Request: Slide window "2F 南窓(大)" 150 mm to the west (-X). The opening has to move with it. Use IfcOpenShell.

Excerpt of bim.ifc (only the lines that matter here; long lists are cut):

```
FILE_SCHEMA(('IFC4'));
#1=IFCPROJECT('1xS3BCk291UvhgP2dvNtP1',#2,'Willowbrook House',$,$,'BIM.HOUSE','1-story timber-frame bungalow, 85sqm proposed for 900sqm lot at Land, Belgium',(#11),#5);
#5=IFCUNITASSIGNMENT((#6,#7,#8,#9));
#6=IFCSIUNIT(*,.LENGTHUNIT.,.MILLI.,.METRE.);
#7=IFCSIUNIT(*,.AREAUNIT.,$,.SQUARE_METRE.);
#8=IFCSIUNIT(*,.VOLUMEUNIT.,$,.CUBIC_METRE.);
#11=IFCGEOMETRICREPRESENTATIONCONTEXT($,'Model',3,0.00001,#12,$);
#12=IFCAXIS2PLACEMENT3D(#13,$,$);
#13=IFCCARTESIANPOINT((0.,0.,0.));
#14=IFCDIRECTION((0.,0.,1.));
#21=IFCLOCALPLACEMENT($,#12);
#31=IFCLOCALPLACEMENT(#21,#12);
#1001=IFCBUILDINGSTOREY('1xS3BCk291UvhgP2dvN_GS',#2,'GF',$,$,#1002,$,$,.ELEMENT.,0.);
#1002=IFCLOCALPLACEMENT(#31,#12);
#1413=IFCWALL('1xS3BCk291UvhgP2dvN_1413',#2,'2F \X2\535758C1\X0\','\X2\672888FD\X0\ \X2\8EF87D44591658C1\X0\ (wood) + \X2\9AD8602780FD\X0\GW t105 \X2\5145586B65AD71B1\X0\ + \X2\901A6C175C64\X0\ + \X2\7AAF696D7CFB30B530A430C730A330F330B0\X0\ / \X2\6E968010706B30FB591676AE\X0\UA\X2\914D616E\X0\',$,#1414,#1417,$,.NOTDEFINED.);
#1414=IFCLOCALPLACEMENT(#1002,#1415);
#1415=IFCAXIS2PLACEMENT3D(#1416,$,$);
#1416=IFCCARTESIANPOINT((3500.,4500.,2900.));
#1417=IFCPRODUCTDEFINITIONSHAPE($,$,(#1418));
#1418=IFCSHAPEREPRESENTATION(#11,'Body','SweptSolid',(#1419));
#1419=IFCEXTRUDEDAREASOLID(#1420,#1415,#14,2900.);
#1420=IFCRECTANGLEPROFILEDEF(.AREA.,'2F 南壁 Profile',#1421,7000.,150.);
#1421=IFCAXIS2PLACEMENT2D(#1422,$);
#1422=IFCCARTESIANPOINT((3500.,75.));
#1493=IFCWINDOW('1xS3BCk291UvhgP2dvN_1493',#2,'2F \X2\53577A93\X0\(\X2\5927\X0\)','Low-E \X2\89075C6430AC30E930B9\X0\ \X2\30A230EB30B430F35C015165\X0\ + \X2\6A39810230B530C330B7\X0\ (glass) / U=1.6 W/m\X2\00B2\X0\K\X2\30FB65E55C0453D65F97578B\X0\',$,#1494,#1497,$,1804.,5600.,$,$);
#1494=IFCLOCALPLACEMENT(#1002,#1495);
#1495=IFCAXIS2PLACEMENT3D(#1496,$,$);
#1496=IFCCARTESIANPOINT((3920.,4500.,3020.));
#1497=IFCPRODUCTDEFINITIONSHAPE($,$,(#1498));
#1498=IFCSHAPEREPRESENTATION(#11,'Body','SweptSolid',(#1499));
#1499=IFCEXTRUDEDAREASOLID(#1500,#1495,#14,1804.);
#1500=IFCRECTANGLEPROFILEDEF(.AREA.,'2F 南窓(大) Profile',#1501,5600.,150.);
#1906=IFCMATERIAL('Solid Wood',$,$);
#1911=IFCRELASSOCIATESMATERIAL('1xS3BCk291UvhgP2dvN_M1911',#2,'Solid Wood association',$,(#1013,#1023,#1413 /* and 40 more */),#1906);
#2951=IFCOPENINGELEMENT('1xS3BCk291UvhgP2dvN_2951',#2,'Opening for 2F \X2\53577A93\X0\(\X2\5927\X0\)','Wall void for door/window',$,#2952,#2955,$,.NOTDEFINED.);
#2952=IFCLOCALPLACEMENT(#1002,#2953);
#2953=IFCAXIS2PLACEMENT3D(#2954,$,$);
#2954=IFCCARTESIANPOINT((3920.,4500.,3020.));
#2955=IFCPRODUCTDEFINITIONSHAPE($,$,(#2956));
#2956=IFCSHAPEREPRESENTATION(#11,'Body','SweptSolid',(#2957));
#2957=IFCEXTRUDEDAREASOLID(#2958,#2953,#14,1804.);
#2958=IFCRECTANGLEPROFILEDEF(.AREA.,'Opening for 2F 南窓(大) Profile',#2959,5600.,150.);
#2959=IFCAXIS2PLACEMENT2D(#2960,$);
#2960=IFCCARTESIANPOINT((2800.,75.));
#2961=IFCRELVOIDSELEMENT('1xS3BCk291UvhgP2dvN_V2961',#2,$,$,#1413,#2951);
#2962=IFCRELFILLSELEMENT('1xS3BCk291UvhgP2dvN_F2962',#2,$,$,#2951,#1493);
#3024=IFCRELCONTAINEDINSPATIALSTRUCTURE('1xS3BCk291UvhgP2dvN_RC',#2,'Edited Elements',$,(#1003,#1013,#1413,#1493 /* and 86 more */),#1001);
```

```python
import ifcopenshell
import ifcopenshell.api.geometry
import ifcopenshell.util.placement

model = ifcopenshell.open("bim.ifc")

window = model.by_guid("1xS3BCk291UvhgP2dvN_1493")
opening = window.FillsVoids[0].RelatingOpeningElement
wall = opening.VoidsElements[0].RelatingBuildingElement

wall_matrix = ifcopenshell.util.placement.get_local_placement(wall.ObjectPlacement)
shift = wall_matrix[:3, 0] * -150.0
before = ifcopenshell.util.placement.get_local_placement(window.ObjectPlacement)[:3, 3].copy()

# The window is not placed relative to its opening, so move both.
for product in (opening, window):
    matrix = ifcopenshell.util.placement.get_local_placement(product.ObjectPlacement)
    matrix[:3, 3] += shift
    ifcopenshell.api.geometry.edit_object_placement(model, product=product, matrix=matrix, is_si=False)

after = ifcopenshell.util.placement.get_local_placement(window.ObjectPlacement)[:3, 3]
print("window moved by", (after - before).round(3) + 0.0)

model.write("bim_rev.ifc")
```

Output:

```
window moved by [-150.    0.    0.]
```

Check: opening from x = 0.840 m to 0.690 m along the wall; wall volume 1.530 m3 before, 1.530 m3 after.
